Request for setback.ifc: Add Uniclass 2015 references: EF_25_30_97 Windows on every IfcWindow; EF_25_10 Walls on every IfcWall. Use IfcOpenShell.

First a look at what the model holds.

```python
import ifcopenshell

model = ifcopenshell.open("setback.ifc")
print(model.schema)
print("classifications:", [c.Name for c in model.by_type("IfcClassification")])
for ifc_class in ("IfcDoor", "IfcRoof", "IfcStair", "IfcWall", "IfcWindow"):
    print(ifc_class, len(model.by_type(ifc_class)))
```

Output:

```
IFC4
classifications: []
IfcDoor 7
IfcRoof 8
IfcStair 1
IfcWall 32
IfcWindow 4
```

```python
import ifcopenshell
import ifcopenshell.api.classification

model = ifcopenshell.open("setback.ifc")

system = ifcopenshell.api.classification.add_classification(model, classification="Uniclass 2015")

codes = {
    "IfcWindow": ("EF_25_30_97", "Windows"),
    "IfcWall": ("EF_25_10", "Walls"),
}
for ifc_class, (code, name) in codes.items():
    products = model.by_type(ifc_class)
    ifcopenshell.api.classification.add_reference(
        model, products=products, classification=system, identification=code, name=name
    )
    print(code, len(products))

model.write("setback_edited.ifc")
```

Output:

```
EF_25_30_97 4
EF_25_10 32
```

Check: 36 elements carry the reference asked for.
